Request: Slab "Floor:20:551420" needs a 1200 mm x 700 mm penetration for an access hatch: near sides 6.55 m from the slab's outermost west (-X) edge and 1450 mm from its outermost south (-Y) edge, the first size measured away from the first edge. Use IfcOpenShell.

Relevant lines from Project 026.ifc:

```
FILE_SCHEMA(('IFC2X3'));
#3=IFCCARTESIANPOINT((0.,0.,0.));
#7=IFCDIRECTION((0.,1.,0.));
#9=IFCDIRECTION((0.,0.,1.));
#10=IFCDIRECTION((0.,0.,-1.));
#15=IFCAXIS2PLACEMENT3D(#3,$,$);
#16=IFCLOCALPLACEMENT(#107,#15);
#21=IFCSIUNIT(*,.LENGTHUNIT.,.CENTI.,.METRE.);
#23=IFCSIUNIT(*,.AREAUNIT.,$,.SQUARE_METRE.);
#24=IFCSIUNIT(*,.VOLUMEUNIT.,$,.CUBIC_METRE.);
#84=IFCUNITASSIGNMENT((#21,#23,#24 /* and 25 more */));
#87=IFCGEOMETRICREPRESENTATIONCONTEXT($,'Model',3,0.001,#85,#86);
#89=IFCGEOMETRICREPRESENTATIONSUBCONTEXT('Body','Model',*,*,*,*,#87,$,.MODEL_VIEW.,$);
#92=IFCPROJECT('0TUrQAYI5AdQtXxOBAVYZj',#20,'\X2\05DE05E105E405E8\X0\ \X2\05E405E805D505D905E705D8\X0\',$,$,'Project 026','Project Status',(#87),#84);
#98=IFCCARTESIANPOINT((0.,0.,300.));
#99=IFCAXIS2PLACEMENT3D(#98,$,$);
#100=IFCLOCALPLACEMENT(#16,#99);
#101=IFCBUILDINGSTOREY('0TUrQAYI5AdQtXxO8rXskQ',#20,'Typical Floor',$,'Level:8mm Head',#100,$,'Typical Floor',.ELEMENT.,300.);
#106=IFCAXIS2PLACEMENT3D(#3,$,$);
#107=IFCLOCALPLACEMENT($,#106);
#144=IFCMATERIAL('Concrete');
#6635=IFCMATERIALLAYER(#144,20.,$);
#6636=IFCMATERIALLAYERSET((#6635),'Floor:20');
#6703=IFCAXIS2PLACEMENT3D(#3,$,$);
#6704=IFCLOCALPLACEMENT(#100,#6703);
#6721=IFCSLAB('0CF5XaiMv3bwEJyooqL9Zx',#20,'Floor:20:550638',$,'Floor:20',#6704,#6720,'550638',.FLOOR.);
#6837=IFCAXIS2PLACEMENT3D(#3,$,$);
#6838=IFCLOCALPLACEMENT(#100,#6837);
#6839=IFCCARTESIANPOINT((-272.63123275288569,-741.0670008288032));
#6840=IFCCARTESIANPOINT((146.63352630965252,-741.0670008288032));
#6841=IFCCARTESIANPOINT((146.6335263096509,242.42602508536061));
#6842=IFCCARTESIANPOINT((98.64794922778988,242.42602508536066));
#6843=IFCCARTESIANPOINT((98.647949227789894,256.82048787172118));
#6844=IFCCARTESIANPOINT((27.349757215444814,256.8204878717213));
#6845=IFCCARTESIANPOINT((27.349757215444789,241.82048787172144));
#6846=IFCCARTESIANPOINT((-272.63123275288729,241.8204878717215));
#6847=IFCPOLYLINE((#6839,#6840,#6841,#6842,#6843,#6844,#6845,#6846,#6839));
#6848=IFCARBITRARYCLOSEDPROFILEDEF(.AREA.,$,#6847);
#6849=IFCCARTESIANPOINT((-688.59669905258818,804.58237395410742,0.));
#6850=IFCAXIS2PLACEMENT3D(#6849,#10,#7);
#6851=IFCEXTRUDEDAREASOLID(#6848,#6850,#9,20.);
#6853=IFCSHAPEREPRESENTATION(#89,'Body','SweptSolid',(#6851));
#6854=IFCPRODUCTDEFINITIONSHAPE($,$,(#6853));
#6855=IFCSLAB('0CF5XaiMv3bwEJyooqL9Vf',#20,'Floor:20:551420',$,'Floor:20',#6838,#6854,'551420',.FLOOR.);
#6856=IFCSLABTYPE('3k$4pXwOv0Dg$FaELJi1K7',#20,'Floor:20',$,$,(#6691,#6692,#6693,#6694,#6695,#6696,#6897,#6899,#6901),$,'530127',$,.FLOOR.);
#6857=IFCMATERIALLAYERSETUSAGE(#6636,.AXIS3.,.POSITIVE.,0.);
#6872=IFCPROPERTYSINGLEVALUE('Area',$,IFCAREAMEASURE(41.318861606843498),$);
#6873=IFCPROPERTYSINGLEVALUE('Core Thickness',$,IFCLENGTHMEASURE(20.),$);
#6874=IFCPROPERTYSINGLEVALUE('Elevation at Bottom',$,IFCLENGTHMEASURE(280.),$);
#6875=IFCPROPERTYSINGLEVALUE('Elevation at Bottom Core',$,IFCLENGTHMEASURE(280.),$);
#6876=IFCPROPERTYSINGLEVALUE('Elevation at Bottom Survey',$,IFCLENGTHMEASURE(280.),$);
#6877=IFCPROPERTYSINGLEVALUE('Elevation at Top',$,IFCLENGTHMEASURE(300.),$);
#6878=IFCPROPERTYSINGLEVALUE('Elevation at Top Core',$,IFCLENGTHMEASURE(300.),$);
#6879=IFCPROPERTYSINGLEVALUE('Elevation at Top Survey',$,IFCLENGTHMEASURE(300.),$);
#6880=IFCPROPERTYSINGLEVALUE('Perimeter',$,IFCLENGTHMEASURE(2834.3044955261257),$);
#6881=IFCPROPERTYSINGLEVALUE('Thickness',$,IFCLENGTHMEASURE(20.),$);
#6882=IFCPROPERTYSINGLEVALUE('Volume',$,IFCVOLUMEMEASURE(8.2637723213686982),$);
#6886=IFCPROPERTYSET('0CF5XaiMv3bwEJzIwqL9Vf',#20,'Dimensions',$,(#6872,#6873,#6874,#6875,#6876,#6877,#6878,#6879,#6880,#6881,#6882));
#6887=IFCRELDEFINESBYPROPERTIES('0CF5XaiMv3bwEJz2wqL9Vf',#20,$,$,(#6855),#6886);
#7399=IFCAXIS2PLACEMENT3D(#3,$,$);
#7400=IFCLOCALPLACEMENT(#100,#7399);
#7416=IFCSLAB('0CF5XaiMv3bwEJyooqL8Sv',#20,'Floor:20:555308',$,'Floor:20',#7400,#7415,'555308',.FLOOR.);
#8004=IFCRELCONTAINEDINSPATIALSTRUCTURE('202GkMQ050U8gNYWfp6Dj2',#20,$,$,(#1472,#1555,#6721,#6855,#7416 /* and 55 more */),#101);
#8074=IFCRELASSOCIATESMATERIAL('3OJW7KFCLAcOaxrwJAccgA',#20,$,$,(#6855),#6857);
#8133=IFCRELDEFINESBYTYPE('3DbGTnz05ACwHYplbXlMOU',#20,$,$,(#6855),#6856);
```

```python
import numpy as np
import ifcopenshell
import ifcopenshell.api.feature
import ifcopenshell.api.geometry
import ifcopenshell.api.pset
import ifcopenshell.api.root
import ifcopenshell.geom
import ifcopenshell.util.element
import ifcopenshell.util.placement
import ifcopenshell.util.representation
import ifcopenshell.util.shape
import ifcopenshell.util.unit

model = ifcopenshell.open("Project 026.ifc")
unit_scale = ifcopenshell.util.unit.calculate_unit_scale(model)
area_scale = ifcopenshell.util.unit.calculate_unit_scale(model, "AREAUNIT")
volume_scale = ifcopenshell.util.unit.calculate_unit_scale(model, "VOLUMEUNIT")
settings = ifcopenshell.geom.settings()


def volume(element):
    """Net volume in cubic metres, openings subtracted."""
    shape = ifcopenshell.geom.create_shape(settings, element)
    return ifcopenshell.util.shape.get_volume(shape.geometry)


slab = model.by_guid("0CF5XaiMv3bwEJyooqL9Vf")
before = volume(slab)

# Extent in the slab's own axes, in metres. The edges named are its -X and -Y sides.
slab_shape = ifcopenshell.geom.create_shape(settings, slab)
vertices = ifcopenshell.util.shape.get_vertices(slab_shape.geometry)
x_min, y_min, bottom = vertices.min(axis=0)
top = vertices[:, 2].max()

opening = ifcopenshell.api.root.create_entity(model, ifc_class="IfcOpeningElement", name="Access hatch opening")
context = ifcopenshell.util.representation.get_context(model, "Model", "Body", "MODEL_VIEW")
width, depth = 1.2, 0.7
outline = [(0.0, 0.0), (width, 0.0), (width, depth), (0.0, depth), (0.0, 0.0)]
# Overshoot both faces by 50 mm so the cut is clean.
shape = ifcopenshell.api.geometry.add_slab_representation(
    model, context=context, depth=top - bottom + 0.1, polyline=outline
)
ifcopenshell.api.geometry.assign_representation(model, product=opening, representation=shape)

matrix = ifcopenshell.util.placement.get_local_placement(slab.ObjectPlacement)
matrix[:, 3] = matrix @ np.append(np.array([x_min + 6.55, y_min + 1.45, bottom - 0.05]) / unit_scale, 1.0)
ifcopenshell.api.geometry.edit_object_placement(model, product=opening, matrix=matrix, is_si=False)
ifcopenshell.api.feature.add_feature(model, feature=opening, element=slab)

after = volume(slab)

# Update the slab's stored quantities.
pset = model.by_id(ifcopenshell.util.element.get_pset(slab, "Dimensions", should_inherit=False)["id"])
ifcopenshell.api.pset.edit_pset(model, pset=pset, properties={
    "Area": model.create_entity("IfcAreaMeasure", after / (top - bottom) / area_scale),
    "Volume": model.create_entity("IfcVolumeMeasure", after / volume_scale),
})

print(f"slab volume {before:.3f} -> {after:.3f} m3")

model.write("Project 026_updated.ifc")
```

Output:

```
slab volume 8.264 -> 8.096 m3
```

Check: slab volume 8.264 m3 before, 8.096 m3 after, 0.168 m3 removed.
